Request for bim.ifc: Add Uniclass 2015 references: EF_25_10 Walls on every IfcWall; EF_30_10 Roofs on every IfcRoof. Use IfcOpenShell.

First a look at what the model holds.

```python
import ifcopenshell

model = ifcopenshell.open("bim.ifc")
print(model.schema)
print("classifications:", [c.Name for c in model.by_type("IfcClassification")])
for ifc_class in ("IfcDoor", "IfcRoof", "IfcStair", "IfcWall", "IfcWindow"):
    print(ifc_class, len(model.by_type(ifc_class)))
```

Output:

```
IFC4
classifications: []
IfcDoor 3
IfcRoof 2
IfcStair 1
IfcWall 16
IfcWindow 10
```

```python
import ifcopenshell
import ifcopenshell.api.classification

model = ifcopenshell.open("bim.ifc")

system = ifcopenshell.api.classification.add_classification(model, classification="Uniclass 2015")

codes = {
    "IfcWall": ("EF_25_10", "Walls"),
    "IfcRoof": ("EF_30_10", "Roofs"),
}
for ifc_class, (code, name) in codes.items():
    products = model.by_type(ifc_class)
    ifcopenshell.api.classification.add_reference(
        model, products=products, classification=system, identification=code, name=name
    )
    print(code, len(products))

model.write("bim_v2.ifc")
```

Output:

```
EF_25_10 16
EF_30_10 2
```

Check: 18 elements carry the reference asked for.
